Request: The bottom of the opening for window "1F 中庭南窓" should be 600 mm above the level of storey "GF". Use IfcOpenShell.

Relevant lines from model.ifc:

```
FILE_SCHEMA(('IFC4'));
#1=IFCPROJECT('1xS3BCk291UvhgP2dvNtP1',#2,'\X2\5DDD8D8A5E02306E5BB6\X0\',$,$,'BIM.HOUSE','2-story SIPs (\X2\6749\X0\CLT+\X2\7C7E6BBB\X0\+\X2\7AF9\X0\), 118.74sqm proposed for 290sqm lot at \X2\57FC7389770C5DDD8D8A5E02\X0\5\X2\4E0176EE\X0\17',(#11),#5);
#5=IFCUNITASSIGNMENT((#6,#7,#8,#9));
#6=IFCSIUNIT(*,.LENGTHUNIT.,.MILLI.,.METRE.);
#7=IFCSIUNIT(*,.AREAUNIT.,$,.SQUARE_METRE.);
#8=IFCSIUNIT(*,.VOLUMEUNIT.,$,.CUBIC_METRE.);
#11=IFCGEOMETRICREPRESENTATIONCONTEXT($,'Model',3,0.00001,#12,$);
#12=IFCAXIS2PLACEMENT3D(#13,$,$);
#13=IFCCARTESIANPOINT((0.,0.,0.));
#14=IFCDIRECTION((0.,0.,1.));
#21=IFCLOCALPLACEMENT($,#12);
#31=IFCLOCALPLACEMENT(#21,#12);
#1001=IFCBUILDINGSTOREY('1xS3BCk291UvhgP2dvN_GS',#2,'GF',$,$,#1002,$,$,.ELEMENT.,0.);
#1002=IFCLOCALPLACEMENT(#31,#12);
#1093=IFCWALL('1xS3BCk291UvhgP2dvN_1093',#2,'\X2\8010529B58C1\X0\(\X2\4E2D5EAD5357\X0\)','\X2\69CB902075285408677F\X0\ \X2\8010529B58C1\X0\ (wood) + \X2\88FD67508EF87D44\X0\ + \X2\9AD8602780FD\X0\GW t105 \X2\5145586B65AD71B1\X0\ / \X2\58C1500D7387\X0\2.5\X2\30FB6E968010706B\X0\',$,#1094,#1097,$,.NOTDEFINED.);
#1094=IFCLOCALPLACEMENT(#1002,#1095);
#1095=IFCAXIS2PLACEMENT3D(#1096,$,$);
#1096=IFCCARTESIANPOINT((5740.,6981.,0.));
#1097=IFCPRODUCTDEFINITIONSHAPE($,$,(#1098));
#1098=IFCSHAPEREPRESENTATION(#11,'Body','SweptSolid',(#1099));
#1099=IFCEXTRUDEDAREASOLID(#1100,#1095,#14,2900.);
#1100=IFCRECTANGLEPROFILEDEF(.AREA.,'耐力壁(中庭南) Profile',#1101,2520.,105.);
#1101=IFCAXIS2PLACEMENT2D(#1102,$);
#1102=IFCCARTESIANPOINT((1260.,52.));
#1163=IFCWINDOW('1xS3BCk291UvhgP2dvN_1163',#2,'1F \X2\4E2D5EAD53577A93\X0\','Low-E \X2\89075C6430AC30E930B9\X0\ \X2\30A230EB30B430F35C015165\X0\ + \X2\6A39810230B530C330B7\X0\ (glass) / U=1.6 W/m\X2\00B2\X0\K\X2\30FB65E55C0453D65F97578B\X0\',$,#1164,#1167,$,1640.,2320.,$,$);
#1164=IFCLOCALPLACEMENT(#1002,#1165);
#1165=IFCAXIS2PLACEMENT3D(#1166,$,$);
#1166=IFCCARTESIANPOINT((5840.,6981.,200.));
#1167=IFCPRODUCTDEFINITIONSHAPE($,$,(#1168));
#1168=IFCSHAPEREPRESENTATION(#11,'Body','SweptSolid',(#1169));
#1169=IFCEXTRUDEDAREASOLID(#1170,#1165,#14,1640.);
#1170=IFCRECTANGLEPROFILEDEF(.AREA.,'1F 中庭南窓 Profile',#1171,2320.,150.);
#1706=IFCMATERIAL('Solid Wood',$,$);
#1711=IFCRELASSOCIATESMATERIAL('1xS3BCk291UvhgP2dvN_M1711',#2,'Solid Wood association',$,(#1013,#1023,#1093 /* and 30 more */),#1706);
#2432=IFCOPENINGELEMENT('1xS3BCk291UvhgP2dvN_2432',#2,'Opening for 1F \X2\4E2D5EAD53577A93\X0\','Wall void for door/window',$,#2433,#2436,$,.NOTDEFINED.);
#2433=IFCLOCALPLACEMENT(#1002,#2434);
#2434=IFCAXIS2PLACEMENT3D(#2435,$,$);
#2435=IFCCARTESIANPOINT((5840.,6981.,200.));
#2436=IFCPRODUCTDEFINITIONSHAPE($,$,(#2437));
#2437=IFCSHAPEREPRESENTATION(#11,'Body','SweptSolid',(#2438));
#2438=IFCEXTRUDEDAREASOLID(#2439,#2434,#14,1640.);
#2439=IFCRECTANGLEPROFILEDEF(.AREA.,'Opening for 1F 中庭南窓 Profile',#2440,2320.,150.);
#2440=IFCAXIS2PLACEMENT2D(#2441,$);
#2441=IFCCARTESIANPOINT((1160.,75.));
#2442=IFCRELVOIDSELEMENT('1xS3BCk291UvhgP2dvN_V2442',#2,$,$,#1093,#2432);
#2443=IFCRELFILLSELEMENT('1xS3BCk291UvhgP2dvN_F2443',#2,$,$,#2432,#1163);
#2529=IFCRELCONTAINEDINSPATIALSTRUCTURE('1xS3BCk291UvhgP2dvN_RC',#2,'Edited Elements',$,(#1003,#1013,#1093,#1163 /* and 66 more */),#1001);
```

```python
import numpy as np
import ifcopenshell
import ifcopenshell.api.geometry
import ifcopenshell.geom
import ifcopenshell.util.element
import ifcopenshell.util.placement
import ifcopenshell.util.shape
import ifcopenshell.util.unit

model = ifcopenshell.open("model.ifc")
unit_scale = ifcopenshell.util.unit.calculate_unit_scale(model)

window = model.by_guid("1xS3BCk291UvhgP2dvN_1163")
opening = window.FillsVoids[0].RelatingOpeningElement
storey = ifcopenshell.util.element.get_container(window, ifc_class="IfcBuildingStorey")
level = ifcopenshell.util.placement.get_local_placement(storey.ObjectPlacement)[2, 3]

# The opening's origin need not be at the sill, so measure its lowest point.
shape = ifcopenshell.geom.create_shape(ifcopenshell.geom.settings(), opening)
bottom = ifcopenshell.util.shape.get_shape_bottom_elevation(shape, shape.geometry) / unit_scale
dz = level + 0.6 / unit_scale - bottom

shift = np.array([0.0, 0.0, dz])
# The window is not placed relative to its opening, so move both.
for product in (opening, window):
    matrix = ifcopenshell.util.placement.get_local_placement(product.ObjectPlacement)
    matrix[:3, 3] += shift
    ifcopenshell.api.geometry.edit_object_placement(model, product=product, matrix=matrix, is_si=False)

print(f"moved by {dz * unit_scale:+.3f} m")

model.write("model-out.ifc")
```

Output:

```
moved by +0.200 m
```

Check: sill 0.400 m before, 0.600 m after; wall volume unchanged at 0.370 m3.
